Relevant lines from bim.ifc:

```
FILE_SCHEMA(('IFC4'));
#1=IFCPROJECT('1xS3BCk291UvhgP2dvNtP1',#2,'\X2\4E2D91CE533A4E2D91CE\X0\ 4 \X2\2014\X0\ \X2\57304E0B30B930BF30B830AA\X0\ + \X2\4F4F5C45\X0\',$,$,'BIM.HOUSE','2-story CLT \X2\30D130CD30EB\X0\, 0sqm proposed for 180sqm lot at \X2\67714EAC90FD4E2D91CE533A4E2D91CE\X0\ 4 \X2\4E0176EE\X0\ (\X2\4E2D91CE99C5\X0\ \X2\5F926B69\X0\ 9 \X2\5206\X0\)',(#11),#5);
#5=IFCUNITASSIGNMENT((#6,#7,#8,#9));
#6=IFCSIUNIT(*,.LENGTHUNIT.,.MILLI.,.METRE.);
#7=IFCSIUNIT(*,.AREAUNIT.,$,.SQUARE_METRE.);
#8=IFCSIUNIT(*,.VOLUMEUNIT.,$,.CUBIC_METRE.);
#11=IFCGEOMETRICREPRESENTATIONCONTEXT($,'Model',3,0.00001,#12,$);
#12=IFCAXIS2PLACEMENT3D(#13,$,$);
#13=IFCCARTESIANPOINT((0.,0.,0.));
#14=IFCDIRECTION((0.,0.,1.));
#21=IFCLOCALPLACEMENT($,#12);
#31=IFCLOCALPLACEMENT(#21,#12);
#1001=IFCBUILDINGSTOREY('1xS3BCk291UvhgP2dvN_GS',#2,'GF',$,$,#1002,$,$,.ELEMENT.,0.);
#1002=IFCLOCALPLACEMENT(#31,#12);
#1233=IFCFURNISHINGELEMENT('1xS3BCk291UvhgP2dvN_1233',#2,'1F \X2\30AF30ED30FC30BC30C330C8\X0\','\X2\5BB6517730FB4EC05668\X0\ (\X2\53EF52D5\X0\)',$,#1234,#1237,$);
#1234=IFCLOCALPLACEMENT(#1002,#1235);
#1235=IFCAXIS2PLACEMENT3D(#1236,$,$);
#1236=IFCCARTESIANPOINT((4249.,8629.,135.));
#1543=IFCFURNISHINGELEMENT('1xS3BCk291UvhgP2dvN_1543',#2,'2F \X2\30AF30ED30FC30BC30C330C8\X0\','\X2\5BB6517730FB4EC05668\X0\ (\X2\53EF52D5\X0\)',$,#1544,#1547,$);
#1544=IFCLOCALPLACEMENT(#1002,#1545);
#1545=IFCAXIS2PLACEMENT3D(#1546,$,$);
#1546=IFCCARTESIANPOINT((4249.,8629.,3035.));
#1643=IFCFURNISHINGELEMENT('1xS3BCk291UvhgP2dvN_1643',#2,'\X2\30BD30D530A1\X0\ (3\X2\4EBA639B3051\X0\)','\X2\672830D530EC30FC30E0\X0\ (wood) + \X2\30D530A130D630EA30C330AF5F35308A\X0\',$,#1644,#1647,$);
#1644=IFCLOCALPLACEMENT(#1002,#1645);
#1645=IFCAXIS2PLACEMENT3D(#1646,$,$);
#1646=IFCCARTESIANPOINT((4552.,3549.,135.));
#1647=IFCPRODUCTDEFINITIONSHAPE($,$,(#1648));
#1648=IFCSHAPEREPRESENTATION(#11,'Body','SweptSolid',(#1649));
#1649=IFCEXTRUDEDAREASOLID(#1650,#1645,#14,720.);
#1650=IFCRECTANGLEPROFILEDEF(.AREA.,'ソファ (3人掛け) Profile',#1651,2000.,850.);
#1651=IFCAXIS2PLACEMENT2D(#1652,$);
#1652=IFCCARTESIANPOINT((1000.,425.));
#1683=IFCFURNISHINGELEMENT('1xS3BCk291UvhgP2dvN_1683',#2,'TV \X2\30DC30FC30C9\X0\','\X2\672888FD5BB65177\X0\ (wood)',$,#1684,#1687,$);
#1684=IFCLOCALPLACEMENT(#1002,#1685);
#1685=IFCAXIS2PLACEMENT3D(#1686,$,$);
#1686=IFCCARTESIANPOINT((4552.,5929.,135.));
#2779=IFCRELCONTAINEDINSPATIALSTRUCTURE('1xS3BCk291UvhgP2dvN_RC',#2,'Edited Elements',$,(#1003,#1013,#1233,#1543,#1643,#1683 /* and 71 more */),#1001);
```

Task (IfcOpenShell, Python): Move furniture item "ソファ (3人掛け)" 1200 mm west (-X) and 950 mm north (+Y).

```python
import ifcopenshell
import ifcopenshell.api.geometry
import ifcopenshell.util.placement
import ifcopenshell.util.unit

model = ifcopenshell.open("bim.ifc")
unit_scale = ifcopenshell.util.unit.calculate_unit_scale(model)

item = model.by_guid("1xS3BCk291UvhgP2dvN_1643")
matrix = ifcopenshell.util.placement.get_local_placement(item.ObjectPlacement)
matrix[0, 3] -= 1.2 / unit_scale
matrix[1, 3] += 0.95 / unit_scale
ifcopenshell.api.geometry.edit_object_placement(model, product=item, matrix=matrix, is_si=False)

print(ifcopenshell.util.placement.get_local_placement(item.ObjectPlacement).round(3) + 0.0)

model.write("bim_edited.ifc")
```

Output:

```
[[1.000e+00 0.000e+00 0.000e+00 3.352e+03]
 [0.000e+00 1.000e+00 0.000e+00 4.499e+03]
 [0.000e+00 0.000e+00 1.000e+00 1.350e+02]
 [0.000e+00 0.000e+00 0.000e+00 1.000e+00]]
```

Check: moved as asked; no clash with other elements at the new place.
